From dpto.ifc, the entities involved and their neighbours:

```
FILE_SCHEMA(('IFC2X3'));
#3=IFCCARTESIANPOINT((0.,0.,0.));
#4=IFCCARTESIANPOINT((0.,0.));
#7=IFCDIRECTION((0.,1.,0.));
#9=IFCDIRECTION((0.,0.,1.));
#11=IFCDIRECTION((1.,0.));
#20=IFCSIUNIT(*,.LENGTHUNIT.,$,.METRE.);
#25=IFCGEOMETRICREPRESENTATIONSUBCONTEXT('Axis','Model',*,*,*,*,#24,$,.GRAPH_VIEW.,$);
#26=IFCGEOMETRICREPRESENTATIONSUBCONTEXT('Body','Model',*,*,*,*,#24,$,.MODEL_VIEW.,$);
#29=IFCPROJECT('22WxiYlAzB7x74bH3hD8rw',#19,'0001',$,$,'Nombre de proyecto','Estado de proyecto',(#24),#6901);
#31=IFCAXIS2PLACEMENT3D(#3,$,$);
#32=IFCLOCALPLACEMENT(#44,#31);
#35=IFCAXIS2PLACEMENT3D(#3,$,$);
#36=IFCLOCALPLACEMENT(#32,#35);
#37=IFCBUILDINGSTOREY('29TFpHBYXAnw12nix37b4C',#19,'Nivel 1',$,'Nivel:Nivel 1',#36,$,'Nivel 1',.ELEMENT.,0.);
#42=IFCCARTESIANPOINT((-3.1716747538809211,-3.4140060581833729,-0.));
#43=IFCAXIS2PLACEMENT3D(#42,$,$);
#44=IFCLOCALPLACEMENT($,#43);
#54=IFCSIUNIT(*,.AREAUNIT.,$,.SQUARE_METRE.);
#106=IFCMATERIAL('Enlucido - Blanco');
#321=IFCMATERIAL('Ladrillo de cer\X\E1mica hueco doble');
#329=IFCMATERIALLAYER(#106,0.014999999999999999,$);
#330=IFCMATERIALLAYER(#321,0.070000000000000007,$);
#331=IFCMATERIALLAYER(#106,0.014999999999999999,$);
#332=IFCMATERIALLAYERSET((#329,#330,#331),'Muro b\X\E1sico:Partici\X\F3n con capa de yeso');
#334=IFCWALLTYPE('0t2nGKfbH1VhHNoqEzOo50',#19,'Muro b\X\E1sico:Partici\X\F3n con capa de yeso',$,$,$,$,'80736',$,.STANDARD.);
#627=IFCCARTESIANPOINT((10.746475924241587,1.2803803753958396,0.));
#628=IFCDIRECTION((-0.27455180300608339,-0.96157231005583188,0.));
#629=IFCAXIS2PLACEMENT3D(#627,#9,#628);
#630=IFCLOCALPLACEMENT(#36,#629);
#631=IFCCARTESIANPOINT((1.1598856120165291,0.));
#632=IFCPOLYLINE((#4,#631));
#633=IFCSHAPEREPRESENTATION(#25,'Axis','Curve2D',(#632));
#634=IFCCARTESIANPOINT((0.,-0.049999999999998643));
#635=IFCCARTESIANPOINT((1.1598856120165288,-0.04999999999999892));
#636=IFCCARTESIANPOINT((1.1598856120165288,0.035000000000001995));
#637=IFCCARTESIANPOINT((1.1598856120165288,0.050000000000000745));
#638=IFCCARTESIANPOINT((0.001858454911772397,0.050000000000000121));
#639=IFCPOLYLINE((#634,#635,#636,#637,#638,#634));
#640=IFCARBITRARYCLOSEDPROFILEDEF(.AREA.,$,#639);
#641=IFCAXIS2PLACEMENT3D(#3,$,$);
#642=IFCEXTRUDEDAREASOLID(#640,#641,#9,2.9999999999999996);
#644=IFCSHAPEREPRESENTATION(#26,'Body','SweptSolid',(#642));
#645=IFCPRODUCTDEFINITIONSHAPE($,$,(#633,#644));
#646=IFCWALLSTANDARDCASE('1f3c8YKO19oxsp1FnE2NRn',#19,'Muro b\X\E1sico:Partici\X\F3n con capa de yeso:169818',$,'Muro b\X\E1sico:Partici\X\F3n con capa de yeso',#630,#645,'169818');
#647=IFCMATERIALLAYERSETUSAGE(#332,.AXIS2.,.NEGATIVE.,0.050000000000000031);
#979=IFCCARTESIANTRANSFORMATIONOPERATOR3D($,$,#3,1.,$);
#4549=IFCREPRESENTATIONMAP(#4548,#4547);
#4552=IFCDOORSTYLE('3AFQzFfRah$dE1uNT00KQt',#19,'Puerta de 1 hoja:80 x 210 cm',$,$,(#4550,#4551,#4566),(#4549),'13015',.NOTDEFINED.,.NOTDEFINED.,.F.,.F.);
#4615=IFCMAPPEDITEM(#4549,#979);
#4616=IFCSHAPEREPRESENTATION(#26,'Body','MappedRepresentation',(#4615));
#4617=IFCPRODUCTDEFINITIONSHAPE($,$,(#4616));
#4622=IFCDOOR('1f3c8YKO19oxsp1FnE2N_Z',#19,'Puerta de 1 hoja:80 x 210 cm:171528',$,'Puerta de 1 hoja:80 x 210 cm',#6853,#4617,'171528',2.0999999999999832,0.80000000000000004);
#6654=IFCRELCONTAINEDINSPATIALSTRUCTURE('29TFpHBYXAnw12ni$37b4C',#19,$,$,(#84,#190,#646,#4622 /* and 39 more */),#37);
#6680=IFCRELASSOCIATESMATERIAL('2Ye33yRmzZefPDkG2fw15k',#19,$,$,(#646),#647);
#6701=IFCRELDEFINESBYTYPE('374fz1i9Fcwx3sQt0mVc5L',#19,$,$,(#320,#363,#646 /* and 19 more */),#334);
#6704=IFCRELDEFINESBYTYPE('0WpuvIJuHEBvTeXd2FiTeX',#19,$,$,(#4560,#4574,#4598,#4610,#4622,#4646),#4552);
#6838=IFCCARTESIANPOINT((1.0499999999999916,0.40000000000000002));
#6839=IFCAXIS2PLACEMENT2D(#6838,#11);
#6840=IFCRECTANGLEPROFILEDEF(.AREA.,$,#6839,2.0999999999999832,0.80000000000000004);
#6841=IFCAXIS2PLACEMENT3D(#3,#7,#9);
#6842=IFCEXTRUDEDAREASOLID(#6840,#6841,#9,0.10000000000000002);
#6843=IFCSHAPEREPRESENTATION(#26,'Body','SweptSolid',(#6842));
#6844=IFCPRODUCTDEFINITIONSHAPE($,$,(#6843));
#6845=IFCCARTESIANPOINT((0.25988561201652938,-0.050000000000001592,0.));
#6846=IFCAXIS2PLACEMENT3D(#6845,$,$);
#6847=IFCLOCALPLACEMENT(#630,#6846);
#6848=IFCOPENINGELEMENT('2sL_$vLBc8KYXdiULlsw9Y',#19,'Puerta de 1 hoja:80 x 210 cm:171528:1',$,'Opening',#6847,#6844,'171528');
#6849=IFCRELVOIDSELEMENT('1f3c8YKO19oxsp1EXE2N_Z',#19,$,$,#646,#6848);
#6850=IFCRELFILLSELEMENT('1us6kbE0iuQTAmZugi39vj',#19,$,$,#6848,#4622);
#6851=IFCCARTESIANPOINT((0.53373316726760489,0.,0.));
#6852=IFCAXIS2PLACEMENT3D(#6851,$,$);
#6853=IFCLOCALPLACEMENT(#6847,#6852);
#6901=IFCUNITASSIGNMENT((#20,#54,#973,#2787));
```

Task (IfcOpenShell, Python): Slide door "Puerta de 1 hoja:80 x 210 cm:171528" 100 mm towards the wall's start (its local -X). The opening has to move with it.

```python
import ifcopenshell
import ifcopenshell.api.geometry
import ifcopenshell.util.placement

model = ifcopenshell.open("dpto.ifc")

door = model.by_guid("1f3c8YKO19oxsp1FnE2N_Z")
opening = door.FillsVoids[0].RelatingOpeningElement
wall = opening.VoidsElements[0].RelatingBuildingElement

wall_matrix = ifcopenshell.util.placement.get_local_placement(wall.ObjectPlacement)
shift = wall_matrix[:3, 0] * -0.1
before = ifcopenshell.util.placement.get_local_placement(door.ObjectPlacement)[:3, 3].copy()

# The door is placed relative to its opening, so it follows when the opening moves.
matrix = ifcopenshell.util.placement.get_local_placement(opening.ObjectPlacement)
matrix[:3, 3] += shift
ifcopenshell.api.geometry.edit_object_placement(
    model, product=opening, matrix=matrix, is_si=False, should_transform_children=True
)

after = ifcopenshell.util.placement.get_local_placement(door.ObjectPlacement)[:3, 3]
print("door moved by", (after - before).round(3) + 0.0)

model.write("dpto_rev.ifc")
```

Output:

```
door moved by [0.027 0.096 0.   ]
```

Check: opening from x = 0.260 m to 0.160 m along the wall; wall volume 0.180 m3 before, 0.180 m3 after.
